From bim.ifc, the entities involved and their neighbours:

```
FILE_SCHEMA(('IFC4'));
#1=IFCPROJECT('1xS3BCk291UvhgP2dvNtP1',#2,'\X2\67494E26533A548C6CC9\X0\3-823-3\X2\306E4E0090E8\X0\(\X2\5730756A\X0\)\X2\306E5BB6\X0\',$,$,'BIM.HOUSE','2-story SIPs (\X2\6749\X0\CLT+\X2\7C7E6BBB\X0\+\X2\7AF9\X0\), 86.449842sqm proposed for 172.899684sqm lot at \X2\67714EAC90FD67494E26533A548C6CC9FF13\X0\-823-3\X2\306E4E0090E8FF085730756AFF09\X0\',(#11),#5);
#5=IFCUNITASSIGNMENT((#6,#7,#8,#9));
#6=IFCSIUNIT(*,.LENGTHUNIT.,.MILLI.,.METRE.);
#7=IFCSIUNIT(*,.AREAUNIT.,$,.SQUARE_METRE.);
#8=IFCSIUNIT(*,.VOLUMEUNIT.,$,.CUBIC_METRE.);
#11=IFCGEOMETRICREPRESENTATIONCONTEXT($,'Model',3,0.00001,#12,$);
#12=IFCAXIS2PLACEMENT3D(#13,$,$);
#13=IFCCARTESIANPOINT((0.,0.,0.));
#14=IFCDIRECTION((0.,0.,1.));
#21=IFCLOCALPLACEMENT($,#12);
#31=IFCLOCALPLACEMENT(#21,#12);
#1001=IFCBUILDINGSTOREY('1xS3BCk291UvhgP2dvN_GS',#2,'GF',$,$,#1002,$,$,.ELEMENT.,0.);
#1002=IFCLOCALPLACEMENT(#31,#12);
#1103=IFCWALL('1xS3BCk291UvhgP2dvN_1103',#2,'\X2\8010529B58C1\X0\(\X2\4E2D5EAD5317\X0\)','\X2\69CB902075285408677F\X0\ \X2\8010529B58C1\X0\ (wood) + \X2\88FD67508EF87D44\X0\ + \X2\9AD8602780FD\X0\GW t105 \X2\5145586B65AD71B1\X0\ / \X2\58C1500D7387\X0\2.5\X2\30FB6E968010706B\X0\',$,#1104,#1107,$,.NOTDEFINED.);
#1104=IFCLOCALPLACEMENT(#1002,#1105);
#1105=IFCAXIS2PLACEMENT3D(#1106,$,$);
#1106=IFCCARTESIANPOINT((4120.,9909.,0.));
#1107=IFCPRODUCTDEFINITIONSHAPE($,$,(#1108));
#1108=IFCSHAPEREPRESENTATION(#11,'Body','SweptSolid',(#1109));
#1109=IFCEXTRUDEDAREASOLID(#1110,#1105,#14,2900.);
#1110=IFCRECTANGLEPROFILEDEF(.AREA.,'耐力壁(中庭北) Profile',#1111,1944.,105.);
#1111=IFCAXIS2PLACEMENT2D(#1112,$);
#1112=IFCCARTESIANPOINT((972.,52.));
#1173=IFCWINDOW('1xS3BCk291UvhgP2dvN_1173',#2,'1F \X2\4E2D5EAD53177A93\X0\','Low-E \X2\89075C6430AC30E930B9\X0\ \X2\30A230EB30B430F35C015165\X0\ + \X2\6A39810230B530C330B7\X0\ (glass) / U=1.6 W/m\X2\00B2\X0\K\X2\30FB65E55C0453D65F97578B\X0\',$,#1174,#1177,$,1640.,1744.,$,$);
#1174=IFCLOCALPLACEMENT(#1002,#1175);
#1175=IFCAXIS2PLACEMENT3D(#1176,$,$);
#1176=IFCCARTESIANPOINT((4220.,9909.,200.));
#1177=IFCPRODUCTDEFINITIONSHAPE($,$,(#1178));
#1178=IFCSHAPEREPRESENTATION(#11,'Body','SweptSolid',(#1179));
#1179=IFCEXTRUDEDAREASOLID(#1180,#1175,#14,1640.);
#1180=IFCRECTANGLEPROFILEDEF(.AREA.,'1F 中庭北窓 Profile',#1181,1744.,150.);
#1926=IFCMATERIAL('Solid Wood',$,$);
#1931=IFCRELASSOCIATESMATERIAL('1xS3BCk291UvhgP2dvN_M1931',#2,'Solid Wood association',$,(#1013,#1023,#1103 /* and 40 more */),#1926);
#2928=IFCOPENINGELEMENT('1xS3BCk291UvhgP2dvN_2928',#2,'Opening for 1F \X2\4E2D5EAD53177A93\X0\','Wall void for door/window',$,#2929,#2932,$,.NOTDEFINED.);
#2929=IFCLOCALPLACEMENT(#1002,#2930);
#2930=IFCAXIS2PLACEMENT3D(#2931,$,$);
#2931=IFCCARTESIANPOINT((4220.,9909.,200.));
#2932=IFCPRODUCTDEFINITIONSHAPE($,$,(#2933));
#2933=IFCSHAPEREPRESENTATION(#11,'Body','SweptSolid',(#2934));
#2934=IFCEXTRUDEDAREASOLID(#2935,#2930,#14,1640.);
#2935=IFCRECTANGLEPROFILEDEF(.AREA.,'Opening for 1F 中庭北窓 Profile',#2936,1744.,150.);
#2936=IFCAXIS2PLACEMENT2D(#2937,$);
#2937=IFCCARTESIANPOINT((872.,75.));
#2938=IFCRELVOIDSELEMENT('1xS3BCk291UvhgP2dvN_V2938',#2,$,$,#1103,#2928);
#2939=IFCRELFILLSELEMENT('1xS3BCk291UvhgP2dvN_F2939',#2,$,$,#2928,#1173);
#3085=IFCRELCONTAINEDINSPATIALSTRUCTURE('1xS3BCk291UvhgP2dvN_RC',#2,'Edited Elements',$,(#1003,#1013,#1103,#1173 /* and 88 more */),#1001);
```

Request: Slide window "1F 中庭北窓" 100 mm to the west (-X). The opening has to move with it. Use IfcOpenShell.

```python
import ifcopenshell
import ifcopenshell.api.geometry
import ifcopenshell.util.placement

model = ifcopenshell.open("bim.ifc")

window = model.by_guid("1xS3BCk291UvhgP2dvN_1173")
opening = window.FillsVoids[0].RelatingOpeningElement
wall = opening.VoidsElements[0].RelatingBuildingElement

wall_matrix = ifcopenshell.util.placement.get_local_placement(wall.ObjectPlacement)
shift = wall_matrix[:3, 0] * -100.0
before = ifcopenshell.util.placement.get_local_placement(window.ObjectPlacement)[:3, 3].copy()

# The window is not placed relative to its opening, so move both.
for product in (opening, window):
    matrix = ifcopenshell.util.placement.get_local_placement(product.ObjectPlacement)
    matrix[:3, 3] += shift
    ifcopenshell.api.geometry.edit_object_placement(model, product=product, matrix=matrix, is_si=False)

after = ifcopenshell.util.placement.get_local_placement(window.ObjectPlacement)[:3, 3]
print("window moved by", (after - before).round(3) + 0.0)

model.write("bim_updated.ifc")
```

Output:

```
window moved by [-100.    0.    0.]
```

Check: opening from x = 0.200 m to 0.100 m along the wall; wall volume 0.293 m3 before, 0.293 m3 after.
